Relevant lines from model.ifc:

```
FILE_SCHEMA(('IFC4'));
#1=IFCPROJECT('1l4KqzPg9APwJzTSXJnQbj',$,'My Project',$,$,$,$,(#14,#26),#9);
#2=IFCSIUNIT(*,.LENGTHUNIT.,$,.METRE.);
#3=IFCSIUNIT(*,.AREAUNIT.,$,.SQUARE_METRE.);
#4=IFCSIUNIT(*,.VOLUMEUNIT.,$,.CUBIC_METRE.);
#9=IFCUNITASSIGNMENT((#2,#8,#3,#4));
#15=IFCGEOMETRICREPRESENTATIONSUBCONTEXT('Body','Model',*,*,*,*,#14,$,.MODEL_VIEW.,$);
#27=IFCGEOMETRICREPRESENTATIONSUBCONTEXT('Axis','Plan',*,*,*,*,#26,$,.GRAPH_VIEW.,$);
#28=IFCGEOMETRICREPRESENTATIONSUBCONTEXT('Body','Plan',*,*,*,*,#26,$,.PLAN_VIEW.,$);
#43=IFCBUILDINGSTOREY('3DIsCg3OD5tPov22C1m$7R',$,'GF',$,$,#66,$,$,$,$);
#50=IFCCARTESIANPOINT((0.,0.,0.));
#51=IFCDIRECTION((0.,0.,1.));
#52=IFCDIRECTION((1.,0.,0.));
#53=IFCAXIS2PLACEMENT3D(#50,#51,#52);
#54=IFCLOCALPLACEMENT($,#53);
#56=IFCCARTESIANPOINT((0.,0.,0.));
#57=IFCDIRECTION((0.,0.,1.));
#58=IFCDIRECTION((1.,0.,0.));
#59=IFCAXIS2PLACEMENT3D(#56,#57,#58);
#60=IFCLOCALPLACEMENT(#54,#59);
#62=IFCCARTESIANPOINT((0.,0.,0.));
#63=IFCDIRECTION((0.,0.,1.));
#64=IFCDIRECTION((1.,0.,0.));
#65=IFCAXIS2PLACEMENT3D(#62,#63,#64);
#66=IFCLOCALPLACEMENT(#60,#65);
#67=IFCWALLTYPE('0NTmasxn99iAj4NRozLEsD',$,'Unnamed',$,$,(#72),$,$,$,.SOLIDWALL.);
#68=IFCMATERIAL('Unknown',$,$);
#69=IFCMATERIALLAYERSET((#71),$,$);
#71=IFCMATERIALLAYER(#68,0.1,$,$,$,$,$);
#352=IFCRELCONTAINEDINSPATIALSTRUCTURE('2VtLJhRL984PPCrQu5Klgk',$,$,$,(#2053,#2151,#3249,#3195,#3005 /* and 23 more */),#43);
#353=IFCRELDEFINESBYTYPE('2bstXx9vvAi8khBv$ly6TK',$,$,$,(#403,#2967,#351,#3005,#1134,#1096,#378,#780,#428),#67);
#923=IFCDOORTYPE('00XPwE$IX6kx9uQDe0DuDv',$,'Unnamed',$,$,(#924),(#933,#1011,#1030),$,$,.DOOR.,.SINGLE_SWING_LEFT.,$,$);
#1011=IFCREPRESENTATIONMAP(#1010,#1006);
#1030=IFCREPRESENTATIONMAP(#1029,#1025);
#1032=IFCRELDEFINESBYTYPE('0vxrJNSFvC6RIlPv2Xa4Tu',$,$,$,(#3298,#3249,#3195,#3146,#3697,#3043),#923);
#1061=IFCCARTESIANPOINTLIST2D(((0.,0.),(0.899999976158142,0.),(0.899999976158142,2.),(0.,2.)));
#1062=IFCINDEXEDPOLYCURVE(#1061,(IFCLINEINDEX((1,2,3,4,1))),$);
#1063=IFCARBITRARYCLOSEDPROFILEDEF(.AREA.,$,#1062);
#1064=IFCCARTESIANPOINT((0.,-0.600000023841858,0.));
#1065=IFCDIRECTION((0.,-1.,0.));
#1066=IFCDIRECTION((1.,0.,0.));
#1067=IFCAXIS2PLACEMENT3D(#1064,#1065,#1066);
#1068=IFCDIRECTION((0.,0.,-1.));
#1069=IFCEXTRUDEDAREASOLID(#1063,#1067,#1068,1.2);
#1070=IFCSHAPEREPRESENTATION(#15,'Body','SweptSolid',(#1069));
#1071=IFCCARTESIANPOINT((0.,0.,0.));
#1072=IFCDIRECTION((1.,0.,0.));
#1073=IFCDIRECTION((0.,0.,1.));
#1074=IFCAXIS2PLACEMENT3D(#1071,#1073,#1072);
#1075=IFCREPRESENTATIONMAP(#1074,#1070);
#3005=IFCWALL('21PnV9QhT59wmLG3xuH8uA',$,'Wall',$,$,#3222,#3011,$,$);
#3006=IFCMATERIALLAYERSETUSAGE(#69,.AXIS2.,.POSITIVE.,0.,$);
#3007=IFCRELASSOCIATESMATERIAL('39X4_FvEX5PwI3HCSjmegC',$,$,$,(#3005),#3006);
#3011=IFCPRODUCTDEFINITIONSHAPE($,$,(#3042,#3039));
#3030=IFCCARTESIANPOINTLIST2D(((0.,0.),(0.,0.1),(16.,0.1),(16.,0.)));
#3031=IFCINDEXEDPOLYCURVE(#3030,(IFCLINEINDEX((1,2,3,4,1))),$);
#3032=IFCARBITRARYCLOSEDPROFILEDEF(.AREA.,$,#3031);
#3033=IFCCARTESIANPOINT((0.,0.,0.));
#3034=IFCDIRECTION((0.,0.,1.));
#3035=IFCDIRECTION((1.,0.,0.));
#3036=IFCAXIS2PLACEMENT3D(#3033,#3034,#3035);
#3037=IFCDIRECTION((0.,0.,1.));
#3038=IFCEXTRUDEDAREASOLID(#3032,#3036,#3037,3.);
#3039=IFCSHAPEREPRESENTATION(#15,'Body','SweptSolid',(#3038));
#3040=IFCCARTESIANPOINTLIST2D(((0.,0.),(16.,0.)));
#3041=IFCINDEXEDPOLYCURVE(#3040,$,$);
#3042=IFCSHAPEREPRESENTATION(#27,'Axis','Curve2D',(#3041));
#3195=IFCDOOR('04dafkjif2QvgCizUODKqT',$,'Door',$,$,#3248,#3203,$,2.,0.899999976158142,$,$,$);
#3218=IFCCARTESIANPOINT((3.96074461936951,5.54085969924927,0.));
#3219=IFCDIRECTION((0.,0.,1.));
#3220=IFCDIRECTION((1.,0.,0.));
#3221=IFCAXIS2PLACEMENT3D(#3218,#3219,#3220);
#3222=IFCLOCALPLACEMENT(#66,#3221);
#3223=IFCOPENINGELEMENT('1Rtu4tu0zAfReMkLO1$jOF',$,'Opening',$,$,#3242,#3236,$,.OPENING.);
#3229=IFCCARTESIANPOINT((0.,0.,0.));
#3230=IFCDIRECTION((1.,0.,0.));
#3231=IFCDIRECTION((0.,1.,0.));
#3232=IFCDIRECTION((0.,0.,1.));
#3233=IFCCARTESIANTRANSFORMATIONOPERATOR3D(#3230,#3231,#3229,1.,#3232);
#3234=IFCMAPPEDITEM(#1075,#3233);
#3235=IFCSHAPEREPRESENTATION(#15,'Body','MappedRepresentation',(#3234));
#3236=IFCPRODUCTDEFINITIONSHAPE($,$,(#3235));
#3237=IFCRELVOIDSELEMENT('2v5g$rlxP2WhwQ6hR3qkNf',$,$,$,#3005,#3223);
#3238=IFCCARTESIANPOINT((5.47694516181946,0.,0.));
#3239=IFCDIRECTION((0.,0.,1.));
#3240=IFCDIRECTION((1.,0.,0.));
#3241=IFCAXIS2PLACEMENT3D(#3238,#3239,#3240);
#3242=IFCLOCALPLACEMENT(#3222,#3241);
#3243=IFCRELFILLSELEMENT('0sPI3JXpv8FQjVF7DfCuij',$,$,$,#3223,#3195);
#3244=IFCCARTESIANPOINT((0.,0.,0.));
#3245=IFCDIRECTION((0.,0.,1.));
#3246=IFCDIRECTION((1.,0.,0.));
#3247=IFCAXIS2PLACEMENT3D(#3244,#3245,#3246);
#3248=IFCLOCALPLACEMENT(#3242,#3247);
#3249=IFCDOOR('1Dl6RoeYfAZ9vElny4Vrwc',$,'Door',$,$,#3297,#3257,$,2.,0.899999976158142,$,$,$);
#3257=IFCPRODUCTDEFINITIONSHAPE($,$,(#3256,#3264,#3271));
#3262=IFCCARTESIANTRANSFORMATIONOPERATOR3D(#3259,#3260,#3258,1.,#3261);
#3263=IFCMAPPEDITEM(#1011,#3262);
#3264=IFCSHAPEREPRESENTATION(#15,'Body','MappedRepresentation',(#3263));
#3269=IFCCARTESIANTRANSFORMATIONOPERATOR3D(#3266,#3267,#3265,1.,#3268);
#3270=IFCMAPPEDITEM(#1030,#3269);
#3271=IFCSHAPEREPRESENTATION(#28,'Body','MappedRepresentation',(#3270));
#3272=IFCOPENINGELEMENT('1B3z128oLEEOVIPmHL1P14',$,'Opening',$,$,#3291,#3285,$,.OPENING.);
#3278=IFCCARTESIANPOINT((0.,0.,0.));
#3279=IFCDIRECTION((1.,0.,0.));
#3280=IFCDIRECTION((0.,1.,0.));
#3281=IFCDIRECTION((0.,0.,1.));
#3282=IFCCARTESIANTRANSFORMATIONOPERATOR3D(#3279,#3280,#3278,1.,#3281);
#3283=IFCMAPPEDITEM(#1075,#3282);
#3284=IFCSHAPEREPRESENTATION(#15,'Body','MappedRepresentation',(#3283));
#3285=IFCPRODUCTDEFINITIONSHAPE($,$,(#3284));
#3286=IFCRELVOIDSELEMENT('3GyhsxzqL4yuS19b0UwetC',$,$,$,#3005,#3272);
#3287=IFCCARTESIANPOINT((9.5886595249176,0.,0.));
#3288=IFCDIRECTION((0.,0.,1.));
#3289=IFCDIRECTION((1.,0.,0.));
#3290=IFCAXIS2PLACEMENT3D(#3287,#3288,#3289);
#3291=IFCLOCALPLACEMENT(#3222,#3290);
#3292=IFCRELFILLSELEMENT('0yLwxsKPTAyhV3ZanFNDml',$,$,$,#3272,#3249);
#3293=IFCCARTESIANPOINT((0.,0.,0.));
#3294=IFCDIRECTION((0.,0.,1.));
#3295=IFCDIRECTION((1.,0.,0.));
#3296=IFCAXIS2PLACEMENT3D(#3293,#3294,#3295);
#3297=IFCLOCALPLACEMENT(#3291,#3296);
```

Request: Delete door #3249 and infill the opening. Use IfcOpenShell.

```python
import ifcopenshell
import ifcopenshell.api.feature
import ifcopenshell.api.root
import ifcopenshell.geom
import ifcopenshell.util.shape

model = ifcopenshell.open("model.ifc")
settings = ifcopenshell.geom.settings()


def volume(element):
    """Net volume in cubic metres, openings subtracted."""
    shape = ifcopenshell.geom.create_shape(settings, element)
    return ifcopenshell.util.shape.get_volume(shape.geometry)


door = model.by_guid("1Dl6RoeYfAZ9vElny4Vrwc")
opening = door.FillsVoids[0].RelatingOpeningElement
wall = opening.VoidsElements[0].RelatingBuildingElement
before = volume(wall)

ifcopenshell.api.root.remove_product(model, product=door)
ifcopenshell.api.feature.remove_feature(model, feature=opening)

after = volume(wall)

print(f"wall volume {before:.3f} -> {after:.3f} m3")

model.write("model_rev.ifc")
```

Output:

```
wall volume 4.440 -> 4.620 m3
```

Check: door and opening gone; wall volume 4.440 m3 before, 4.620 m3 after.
